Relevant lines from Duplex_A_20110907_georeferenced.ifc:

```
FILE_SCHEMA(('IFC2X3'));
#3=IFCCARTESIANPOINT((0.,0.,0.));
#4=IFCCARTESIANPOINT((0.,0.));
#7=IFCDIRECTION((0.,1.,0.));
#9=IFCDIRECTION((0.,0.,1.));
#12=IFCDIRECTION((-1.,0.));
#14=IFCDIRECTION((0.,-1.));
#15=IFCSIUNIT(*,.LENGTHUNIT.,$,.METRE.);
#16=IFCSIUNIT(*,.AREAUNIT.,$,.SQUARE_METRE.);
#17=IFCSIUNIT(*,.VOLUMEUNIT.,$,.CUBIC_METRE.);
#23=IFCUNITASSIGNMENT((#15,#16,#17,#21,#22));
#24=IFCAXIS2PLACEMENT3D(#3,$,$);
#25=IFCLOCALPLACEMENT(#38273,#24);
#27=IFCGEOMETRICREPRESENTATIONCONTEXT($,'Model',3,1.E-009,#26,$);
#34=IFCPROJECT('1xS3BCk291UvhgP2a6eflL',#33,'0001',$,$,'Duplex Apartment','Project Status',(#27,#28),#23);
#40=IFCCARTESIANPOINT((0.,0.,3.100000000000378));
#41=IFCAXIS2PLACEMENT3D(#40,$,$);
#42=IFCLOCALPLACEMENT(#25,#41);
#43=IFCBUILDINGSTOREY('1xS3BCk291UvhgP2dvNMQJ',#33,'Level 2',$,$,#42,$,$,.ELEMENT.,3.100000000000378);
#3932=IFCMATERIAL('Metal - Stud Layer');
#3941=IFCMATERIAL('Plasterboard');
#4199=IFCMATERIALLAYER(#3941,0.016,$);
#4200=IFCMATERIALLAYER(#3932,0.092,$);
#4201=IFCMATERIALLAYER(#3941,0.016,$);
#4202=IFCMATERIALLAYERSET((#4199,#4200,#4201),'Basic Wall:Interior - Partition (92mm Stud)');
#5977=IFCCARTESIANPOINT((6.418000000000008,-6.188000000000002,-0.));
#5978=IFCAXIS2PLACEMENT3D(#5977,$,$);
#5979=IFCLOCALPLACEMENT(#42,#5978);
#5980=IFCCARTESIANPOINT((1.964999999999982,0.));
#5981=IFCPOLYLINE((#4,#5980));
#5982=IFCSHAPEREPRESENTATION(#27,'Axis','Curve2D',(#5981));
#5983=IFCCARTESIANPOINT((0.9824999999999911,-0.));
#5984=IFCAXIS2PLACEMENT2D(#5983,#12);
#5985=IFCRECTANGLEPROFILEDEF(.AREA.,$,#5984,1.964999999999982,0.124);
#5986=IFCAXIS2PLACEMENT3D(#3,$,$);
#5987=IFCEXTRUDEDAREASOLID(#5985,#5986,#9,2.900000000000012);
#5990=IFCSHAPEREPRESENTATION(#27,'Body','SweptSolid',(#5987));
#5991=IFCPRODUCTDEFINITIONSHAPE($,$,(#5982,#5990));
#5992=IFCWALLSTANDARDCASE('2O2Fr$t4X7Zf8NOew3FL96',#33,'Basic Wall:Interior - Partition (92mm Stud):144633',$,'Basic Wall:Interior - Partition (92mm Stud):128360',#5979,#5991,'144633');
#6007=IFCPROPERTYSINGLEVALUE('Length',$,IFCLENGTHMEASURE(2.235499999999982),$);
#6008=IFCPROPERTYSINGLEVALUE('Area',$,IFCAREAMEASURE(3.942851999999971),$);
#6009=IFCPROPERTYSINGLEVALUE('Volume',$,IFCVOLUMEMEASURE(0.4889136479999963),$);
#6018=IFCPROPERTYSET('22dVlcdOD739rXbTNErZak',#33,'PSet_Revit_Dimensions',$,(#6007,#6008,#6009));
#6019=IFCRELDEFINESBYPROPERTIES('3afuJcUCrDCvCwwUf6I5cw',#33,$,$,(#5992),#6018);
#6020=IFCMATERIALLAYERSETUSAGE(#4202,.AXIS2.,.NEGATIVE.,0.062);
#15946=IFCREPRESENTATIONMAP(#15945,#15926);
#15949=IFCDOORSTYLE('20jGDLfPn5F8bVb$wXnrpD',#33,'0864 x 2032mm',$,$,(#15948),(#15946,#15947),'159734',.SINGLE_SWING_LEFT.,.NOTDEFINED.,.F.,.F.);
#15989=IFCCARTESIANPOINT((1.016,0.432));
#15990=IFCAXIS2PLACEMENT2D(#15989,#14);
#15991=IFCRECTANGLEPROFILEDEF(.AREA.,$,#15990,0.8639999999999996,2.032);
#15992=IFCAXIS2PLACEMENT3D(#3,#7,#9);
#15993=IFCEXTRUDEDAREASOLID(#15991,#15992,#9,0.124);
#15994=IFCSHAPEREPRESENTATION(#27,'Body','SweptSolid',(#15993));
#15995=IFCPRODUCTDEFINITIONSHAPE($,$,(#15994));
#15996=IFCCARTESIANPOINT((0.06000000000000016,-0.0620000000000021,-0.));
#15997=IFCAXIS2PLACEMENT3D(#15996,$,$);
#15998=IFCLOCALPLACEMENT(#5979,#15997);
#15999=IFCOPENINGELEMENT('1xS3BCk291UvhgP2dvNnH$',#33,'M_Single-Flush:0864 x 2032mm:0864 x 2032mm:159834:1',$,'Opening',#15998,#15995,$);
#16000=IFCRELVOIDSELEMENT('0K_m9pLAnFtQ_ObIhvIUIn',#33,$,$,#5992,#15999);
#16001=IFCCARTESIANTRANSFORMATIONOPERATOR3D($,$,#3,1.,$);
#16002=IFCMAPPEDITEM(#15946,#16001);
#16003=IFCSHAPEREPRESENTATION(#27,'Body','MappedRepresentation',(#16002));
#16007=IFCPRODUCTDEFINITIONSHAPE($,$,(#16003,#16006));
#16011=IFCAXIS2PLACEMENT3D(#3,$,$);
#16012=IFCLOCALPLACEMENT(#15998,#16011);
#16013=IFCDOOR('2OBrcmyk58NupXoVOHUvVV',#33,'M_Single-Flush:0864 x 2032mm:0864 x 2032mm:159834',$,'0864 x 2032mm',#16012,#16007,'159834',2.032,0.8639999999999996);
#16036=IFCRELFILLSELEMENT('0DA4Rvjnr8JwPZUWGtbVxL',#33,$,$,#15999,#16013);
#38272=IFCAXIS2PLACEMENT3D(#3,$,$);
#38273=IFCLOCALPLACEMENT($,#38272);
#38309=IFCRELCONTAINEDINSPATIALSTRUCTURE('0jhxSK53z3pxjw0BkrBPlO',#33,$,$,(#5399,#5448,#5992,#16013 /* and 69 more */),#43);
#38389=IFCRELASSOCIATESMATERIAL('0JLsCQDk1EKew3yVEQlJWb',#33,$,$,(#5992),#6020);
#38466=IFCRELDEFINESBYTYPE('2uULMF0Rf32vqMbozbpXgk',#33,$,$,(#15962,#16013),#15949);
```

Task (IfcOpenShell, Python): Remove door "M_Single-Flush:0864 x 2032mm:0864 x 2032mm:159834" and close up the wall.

```python
import ifcopenshell
import ifcopenshell.api.feature
import ifcopenshell.api.pset
import ifcopenshell.api.root
import ifcopenshell.geom
import ifcopenshell.util.element
import ifcopenshell.util.shape
import ifcopenshell.util.unit

model = ifcopenshell.open("Duplex_A_20110907_georeferenced.ifc")
area_scale = ifcopenshell.util.unit.calculate_unit_scale(model, "AREAUNIT")
volume_scale = ifcopenshell.util.unit.calculate_unit_scale(model, "VOLUMEUNIT")
settings = ifcopenshell.geom.settings()


def volume(element):
    """Net volume in cubic metres, openings subtracted."""
    shape = ifcopenshell.geom.create_shape(settings, element)
    return ifcopenshell.util.shape.get_volume(shape.geometry)


door = model.by_guid("2OBrcmyk58NupXoVOHUvVV")
opening = door.FillsVoids[0].RelatingOpeningElement
wall = opening.VoidsElements[0].RelatingBuildingElement
before = volume(wall)

ifcopenshell.api.root.remove_product(model, product=door)
ifcopenshell.api.feature.remove_feature(model, feature=opening)

after = volume(wall)
thickness = 0.124  # wall thickness in metres

# Update the wall's stored quantities.
pset = model.by_id(ifcopenshell.util.element.get_pset(wall, "PSet_Revit_Dimensions", should_inherit=False)["id"])
ifcopenshell.api.pset.edit_pset(model, pset=pset, properties={
    "Area": model.create_entity("IfcAreaMeasure", after / thickness / area_scale),
    "Volume": model.create_entity("IfcVolumeMeasure", after / volume_scale),
})

print(f"wall volume {before:.3f} -> {after:.3f} m3")

model.write("Duplex_A_20110907_georeferenced_rev.ifc")
```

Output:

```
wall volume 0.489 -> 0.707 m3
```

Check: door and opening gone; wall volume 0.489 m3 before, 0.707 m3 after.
